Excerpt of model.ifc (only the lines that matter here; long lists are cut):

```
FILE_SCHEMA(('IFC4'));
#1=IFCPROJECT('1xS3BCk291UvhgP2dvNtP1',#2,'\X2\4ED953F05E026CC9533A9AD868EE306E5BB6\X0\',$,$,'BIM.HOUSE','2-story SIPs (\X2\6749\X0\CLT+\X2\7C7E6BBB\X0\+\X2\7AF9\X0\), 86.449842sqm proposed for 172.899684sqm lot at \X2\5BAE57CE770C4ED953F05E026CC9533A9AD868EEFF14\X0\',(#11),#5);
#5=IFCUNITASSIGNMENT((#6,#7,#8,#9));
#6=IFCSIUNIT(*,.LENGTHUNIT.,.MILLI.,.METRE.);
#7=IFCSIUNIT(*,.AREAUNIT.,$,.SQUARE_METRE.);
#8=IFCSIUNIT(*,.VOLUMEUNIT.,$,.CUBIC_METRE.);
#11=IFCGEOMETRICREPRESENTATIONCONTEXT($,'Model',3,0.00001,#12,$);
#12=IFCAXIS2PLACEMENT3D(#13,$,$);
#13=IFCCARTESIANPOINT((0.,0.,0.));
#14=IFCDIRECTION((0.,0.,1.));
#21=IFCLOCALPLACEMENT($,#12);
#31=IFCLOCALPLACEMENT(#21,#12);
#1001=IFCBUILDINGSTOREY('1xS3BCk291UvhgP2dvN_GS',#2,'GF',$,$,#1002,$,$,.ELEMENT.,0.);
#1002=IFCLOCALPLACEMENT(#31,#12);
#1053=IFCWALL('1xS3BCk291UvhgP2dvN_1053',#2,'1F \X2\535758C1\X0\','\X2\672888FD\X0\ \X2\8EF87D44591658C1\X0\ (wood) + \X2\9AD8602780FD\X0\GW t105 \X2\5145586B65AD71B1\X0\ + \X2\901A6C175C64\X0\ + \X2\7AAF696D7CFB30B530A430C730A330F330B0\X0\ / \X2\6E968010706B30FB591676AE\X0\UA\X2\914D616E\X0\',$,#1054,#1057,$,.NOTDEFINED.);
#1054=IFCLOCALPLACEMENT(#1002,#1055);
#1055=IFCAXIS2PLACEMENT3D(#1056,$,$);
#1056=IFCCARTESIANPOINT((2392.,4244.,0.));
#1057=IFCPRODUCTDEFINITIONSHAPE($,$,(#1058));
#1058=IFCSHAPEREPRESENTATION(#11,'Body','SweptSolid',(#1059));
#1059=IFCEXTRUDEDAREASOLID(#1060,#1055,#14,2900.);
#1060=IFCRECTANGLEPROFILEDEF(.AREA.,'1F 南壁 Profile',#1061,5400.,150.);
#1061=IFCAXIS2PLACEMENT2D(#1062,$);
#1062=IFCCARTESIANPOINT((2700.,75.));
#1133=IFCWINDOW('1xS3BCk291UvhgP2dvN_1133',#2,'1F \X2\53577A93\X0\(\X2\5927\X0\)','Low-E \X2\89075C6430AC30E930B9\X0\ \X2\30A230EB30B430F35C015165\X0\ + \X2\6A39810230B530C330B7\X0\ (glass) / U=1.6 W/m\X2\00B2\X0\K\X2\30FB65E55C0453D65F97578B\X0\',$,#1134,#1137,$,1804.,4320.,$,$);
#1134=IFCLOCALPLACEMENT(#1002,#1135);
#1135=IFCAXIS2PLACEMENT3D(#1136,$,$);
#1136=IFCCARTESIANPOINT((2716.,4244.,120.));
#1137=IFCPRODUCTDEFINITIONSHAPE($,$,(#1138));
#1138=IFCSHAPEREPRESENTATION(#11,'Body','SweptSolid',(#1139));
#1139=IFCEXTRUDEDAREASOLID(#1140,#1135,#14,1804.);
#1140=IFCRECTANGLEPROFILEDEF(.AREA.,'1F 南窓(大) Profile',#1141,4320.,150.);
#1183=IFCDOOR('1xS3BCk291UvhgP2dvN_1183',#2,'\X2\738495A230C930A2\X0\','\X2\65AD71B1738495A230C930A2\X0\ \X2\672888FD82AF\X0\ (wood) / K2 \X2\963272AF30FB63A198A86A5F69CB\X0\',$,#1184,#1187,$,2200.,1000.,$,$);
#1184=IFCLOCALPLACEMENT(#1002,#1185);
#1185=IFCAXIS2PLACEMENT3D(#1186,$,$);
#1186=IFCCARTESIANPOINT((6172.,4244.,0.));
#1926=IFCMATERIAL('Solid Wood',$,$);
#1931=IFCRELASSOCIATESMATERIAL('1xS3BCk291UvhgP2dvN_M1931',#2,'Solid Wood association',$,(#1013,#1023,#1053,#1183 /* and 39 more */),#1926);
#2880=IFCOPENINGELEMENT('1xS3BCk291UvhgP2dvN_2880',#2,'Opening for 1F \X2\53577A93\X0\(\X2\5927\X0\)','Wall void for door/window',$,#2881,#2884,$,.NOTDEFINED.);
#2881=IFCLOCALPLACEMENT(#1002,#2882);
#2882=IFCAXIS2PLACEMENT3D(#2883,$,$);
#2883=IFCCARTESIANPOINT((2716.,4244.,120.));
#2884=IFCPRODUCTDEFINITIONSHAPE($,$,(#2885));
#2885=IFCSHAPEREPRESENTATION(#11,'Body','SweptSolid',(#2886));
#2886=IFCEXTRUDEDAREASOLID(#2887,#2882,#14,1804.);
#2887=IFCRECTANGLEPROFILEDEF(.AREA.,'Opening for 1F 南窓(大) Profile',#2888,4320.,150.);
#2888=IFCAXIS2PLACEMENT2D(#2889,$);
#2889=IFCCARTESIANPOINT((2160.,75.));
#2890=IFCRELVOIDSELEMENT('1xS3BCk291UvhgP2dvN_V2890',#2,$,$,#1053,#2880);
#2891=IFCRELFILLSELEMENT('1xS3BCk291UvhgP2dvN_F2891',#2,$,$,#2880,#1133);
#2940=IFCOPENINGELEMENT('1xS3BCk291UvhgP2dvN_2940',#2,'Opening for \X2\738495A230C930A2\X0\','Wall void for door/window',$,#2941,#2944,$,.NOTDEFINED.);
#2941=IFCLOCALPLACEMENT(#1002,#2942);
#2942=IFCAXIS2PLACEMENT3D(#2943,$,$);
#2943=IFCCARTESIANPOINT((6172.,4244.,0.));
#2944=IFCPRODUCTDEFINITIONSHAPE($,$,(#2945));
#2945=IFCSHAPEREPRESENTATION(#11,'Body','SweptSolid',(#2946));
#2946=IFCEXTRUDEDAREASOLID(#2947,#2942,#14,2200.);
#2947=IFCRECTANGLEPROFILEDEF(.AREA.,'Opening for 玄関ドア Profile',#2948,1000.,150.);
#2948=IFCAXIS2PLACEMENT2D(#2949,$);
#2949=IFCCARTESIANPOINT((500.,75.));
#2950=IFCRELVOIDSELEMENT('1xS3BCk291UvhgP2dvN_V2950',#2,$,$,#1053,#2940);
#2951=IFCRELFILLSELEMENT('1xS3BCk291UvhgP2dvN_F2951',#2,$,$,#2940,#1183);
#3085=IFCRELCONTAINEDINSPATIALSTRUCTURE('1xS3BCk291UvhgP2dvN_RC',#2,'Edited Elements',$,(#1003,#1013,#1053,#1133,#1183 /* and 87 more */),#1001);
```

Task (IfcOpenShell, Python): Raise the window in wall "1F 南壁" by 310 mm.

```python
import numpy as np
import ifcopenshell
import ifcopenshell.api.geometry
import ifcopenshell.util.placement
import ifcopenshell.util.unit

model = ifcopenshell.open("model.ifc")
unit_scale = ifcopenshell.util.unit.calculate_unit_scale(model)

window = model.by_guid("1xS3BCk291UvhgP2dvN_1133")
opening = window.FillsVoids[0].RelatingOpeningElement
dz = 0.31 / unit_scale

shift = np.array([0.0, 0.0, dz])
# The window is not placed relative to its opening, so move both.
for product in (opening, window):
    matrix = ifcopenshell.util.placement.get_local_placement(product.ObjectPlacement)
    matrix[:3, 3] += shift
    ifcopenshell.api.geometry.edit_object_placement(model, product=product, matrix=matrix, is_si=False)

print(f"moved by {dz * unit_scale:+.3f} m")

model.write("model_v2.ifc")
```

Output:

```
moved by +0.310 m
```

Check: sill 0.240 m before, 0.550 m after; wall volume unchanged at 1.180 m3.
